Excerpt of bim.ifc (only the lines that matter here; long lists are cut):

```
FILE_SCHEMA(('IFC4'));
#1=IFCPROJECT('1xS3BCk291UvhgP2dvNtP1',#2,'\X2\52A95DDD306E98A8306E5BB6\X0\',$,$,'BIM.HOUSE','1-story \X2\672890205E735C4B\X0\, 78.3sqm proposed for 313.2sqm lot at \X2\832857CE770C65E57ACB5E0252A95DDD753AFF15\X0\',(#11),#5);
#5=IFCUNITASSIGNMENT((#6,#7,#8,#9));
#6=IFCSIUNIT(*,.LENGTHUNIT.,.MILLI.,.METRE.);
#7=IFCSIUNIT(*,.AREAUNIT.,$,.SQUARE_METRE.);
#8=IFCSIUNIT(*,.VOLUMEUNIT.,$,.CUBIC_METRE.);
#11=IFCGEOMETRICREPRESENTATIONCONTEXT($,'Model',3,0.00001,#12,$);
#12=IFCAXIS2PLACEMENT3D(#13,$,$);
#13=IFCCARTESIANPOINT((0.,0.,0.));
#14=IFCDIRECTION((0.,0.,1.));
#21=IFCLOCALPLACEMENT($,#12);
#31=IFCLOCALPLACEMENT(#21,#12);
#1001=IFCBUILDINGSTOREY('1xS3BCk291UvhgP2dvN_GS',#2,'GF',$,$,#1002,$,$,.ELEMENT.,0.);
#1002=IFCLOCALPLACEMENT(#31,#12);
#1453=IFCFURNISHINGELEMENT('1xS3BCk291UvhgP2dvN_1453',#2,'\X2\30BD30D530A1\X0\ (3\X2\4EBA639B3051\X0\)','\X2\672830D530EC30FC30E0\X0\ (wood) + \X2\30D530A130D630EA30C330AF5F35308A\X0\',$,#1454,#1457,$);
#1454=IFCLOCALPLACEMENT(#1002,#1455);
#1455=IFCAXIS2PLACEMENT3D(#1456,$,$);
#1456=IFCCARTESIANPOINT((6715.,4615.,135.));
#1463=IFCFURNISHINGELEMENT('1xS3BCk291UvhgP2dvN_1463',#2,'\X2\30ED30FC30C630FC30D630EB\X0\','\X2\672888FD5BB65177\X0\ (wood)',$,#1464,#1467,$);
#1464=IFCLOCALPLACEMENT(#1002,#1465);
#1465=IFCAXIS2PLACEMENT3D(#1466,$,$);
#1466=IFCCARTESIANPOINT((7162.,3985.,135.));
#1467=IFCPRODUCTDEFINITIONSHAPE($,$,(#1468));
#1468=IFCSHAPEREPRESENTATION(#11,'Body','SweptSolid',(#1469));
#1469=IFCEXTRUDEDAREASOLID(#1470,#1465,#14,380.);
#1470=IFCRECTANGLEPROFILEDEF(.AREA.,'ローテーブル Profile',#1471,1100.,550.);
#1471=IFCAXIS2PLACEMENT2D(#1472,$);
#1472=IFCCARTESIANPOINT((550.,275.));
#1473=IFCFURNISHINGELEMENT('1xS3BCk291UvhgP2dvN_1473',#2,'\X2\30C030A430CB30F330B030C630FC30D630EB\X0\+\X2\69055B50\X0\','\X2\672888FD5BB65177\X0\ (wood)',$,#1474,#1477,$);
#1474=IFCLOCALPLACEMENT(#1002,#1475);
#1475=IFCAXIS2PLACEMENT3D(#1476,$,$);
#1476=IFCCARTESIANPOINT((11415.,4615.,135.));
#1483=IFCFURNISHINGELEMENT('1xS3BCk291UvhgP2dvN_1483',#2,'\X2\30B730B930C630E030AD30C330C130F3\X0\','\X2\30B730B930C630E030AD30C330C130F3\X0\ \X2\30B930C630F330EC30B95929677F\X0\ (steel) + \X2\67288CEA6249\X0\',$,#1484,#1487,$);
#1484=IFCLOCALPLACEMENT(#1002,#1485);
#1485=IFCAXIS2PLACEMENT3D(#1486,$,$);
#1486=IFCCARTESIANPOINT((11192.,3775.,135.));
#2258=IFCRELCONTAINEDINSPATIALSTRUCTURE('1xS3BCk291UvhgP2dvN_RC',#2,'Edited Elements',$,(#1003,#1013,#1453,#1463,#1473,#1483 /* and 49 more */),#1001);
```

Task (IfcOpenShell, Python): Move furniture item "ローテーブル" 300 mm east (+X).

```python
import ifcopenshell
import ifcopenshell.api.geometry
import ifcopenshell.util.placement
import ifcopenshell.util.unit

model = ifcopenshell.open("bim.ifc")
unit_scale = ifcopenshell.util.unit.calculate_unit_scale(model)

item = model.by_guid("1xS3BCk291UvhgP2dvN_1463")
matrix = ifcopenshell.util.placement.get_local_placement(item.ObjectPlacement)
matrix[0, 3] += 0.3 / unit_scale
ifcopenshell.api.geometry.edit_object_placement(model, product=item, matrix=matrix, is_si=False)

print(ifcopenshell.util.placement.get_local_placement(item.ObjectPlacement).round(3) + 0.0)

model.write("bim_updated.ifc")
```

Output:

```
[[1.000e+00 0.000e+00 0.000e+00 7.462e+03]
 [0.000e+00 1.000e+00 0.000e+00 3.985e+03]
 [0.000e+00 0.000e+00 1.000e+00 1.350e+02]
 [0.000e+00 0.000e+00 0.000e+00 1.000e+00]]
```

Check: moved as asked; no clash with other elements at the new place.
